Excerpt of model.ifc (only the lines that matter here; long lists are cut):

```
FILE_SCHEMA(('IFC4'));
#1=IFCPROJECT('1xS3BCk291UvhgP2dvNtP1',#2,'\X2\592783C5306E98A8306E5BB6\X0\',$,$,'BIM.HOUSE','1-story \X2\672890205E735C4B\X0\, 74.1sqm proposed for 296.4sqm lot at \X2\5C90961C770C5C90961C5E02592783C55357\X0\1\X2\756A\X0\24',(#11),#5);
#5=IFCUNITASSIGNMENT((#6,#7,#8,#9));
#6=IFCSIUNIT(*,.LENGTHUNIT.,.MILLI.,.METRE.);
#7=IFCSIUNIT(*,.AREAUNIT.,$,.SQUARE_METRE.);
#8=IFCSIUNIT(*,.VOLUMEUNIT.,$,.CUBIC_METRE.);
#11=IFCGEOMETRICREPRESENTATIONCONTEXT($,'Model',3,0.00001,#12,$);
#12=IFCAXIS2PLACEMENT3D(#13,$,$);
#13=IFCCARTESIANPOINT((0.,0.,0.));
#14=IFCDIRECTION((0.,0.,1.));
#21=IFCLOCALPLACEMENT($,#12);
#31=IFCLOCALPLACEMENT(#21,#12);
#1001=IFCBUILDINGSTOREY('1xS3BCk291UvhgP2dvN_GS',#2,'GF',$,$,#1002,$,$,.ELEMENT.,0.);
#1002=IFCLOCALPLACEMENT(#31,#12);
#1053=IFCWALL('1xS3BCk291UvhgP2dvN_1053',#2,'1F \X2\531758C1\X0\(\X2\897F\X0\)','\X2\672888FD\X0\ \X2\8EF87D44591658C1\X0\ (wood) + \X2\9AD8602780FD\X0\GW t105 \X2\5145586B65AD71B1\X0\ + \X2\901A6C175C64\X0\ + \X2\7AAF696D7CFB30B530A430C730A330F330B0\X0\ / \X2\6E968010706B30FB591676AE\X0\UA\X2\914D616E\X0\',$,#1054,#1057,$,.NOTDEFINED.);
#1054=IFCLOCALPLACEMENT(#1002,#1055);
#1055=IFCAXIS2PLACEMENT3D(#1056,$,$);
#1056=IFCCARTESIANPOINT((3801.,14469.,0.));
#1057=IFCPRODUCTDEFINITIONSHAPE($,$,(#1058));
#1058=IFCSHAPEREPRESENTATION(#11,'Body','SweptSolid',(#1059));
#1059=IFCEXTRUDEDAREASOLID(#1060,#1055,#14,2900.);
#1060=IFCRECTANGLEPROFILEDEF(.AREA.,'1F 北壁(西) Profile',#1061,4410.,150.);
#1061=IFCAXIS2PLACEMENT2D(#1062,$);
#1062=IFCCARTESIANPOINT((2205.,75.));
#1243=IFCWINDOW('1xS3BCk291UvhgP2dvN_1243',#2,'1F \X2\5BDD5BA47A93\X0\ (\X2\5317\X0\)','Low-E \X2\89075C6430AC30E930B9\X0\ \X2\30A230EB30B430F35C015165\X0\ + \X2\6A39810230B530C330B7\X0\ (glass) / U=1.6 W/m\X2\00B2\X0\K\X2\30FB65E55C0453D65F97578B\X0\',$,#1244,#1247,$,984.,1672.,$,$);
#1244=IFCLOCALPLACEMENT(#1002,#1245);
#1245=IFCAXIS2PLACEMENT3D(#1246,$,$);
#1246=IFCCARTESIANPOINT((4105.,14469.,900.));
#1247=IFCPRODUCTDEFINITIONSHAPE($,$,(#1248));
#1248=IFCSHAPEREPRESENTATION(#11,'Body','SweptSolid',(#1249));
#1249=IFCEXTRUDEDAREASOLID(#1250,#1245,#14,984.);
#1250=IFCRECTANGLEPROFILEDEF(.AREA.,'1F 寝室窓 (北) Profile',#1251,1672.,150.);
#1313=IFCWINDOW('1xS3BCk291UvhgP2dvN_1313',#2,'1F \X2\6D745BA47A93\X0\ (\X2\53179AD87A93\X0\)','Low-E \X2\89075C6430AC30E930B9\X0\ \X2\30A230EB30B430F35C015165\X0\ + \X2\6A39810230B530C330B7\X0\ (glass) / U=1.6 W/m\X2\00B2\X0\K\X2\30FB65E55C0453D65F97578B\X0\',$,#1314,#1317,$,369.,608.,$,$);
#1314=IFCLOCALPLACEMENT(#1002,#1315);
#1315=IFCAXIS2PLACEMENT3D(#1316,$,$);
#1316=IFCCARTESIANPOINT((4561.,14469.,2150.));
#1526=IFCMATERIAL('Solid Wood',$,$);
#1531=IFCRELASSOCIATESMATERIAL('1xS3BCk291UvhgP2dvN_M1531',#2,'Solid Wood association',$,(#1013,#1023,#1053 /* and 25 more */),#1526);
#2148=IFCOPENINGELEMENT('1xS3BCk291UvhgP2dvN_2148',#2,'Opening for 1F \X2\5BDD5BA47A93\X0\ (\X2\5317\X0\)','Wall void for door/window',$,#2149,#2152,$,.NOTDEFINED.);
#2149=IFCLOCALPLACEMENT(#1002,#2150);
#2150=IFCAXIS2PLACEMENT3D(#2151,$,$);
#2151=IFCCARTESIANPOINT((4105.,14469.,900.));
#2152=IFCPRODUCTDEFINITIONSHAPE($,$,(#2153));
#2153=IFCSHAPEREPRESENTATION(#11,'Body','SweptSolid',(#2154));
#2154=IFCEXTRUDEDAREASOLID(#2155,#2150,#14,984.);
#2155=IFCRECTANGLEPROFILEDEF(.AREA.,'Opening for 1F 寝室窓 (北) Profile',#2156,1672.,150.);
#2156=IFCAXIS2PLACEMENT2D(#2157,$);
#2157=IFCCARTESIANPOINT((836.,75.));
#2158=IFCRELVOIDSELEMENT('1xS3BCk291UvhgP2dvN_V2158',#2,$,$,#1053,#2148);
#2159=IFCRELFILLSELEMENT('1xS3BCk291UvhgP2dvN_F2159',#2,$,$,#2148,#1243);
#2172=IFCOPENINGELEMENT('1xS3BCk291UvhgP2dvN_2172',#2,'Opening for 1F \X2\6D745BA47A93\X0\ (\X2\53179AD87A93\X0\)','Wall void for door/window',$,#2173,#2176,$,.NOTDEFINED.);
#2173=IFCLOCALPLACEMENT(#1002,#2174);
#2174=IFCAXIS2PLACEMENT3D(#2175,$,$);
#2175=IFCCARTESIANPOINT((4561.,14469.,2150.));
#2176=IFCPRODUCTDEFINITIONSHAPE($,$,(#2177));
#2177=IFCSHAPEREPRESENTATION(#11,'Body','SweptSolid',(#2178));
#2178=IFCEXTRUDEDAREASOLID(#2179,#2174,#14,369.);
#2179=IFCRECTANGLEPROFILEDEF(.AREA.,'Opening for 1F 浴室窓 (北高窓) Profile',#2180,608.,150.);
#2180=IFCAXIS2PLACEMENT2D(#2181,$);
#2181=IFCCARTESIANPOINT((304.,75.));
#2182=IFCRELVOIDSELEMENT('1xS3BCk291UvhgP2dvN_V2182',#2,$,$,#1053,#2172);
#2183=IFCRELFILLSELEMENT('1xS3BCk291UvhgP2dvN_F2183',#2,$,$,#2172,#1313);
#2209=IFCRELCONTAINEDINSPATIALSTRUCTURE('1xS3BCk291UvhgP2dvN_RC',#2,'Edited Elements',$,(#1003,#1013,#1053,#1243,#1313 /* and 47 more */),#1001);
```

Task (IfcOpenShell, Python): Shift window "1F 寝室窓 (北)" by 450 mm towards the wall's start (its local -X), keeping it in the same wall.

```python
import ifcopenshell
import ifcopenshell.api.geometry
import ifcopenshell.util.placement

model = ifcopenshell.open("model.ifc")

window = model.by_id(1243)
opening = window.FillsVoids[0].RelatingOpeningElement
wall = opening.VoidsElements[0].RelatingBuildingElement

wall_matrix = ifcopenshell.util.placement.get_local_placement(wall.ObjectPlacement)
shift = wall_matrix[:3, 0] * -450.0
before = ifcopenshell.util.placement.get_local_placement(window.ObjectPlacement)[:3, 3].copy()

# The window is not placed relative to its opening, so move both.
for product in (opening, window):
    matrix = ifcopenshell.util.placement.get_local_placement(product.ObjectPlacement)
    matrix[:3, 3] += shift
    ifcopenshell.api.geometry.edit_object_placement(model, product=product, matrix=matrix, is_si=False)

after = ifcopenshell.util.placement.get_local_placement(window.ObjectPlacement)[:3, 3]
print("window moved by", (after - before).round(3) + 0.0)

model.write("model_edited.ifc")
```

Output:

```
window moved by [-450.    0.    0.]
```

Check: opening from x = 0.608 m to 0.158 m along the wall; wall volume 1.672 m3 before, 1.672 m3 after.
